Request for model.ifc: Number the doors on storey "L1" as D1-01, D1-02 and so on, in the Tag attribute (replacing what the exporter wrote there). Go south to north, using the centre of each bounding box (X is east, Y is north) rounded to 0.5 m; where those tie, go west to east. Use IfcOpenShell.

First a look at what the model holds.

```python
import ifcopenshell
import ifcopenshell.util.element
import ifcopenshell.util.placement

model = ifcopenshell.open("model.ifc")
print(model.schema)
storey = next(s for s in model.by_type("IfcBuildingStorey") if s.Name == "L1")
doors = [e for e in ifcopenshell.util.element.get_decomposition(storey) if e.is_a("IfcDoor")]
for e in sorted(doors, key=lambda e: e.id()):
    origin = ifcopenshell.util.placement.get_local_placement(e.ObjectPlacement)[:3, 3]
    print(e.id(), e.Tag, e.Name, origin.round(2) + 0.0, sep=" | ")
```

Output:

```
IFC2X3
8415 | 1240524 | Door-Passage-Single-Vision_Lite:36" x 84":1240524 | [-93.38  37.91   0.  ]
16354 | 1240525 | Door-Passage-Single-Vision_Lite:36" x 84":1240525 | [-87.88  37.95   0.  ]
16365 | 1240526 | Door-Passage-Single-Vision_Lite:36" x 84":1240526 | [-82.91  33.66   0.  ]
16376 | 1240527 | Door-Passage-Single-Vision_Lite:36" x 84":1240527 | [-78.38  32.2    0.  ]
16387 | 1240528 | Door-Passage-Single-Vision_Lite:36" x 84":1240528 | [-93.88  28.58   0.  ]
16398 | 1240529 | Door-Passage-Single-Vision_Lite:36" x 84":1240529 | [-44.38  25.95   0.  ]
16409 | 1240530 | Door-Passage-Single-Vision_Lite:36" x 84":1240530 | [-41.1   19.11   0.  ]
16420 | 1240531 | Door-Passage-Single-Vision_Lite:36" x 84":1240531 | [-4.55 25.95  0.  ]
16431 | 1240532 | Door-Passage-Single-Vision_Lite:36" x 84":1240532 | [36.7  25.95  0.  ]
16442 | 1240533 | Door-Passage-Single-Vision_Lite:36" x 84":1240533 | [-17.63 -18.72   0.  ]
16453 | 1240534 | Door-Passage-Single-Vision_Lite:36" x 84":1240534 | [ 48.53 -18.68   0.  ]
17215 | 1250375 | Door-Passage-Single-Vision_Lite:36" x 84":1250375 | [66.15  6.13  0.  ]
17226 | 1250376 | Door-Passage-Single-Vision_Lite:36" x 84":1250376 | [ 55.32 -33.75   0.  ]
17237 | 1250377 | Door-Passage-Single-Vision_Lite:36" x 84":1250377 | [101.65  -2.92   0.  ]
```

```python
import ifcopenshell
import ifcopenshell.geom
import ifcopenshell.util.element
import ifcopenshell.util.shape

model = ifcopenshell.open("model.ifc")
settings = ifcopenshell.geom.settings()
settings.set("use-world-coords", True)


def centre(element):
    shape = ifcopenshell.geom.create_shape(settings, element)
    return ifcopenshell.util.shape.get_bbox_centroid(shape.geometry)


storey = next(s for s in model.by_type("IfcBuildingStorey") if s.Name == "L1")
doors = [e for e in ifcopenshell.util.element.get_decomposition(storey) if e.is_a("IfcDoor")]

# Insertion points can sit at a corner or the storey origin, so sort by the geometry (in metres).
centres = {e: centre(e) for e in doors}
doors.sort(key=lambda e: (round(centres[e][1] / 0.5), centres[e][0]))

for i, e in enumerate(doors, start=1):
    number = f"D1-{i:02d}"
    e.Tag = number
    print(e.id(), number)

model.write("model_edited.ifc")
```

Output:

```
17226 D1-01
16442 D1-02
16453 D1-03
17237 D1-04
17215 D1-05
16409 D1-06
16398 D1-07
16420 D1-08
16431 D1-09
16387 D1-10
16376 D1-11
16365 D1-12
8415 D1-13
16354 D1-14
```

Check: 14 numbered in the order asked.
